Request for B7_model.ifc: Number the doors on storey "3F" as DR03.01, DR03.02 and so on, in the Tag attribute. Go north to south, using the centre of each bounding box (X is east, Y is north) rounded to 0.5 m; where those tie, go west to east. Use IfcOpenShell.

First a look at what the model holds.

```python
import ifcopenshell
import ifcopenshell.util.element
import ifcopenshell.util.placement

model = ifcopenshell.open("B7_model.ifc")
print(model.schema)
storey = next(s for s in model.by_type("IfcBuildingStorey") if s.Name == "3F")
doors = [e for e in ifcopenshell.util.element.get_decomposition(storey) if e.is_a("IfcDoor")]
for e in sorted(doors, key=lambda e: e.id()):
    origin = ifcopenshell.util.placement.get_local_placement(e.ObjectPlacement)[:3, 3]
    print(e.id(), e.Tag, e.Name, origin.round(2) + 0.0, sep=" | ")
```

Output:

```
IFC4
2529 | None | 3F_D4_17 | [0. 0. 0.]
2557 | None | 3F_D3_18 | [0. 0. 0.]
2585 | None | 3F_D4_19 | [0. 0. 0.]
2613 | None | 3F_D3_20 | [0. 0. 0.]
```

```python
import ifcopenshell
import ifcopenshell.geom
import ifcopenshell.util.element
import ifcopenshell.util.shape

model = ifcopenshell.open("B7_model.ifc")
settings = ifcopenshell.geom.settings()
settings.set("use-world-coords", True)


def centre(element):
    shape = ifcopenshell.geom.create_shape(settings, element)
    return ifcopenshell.util.shape.get_bbox_centroid(shape.geometry)


storey = next(s for s in model.by_type("IfcBuildingStorey") if s.Name == "3F")
doors = [e for e in ifcopenshell.util.element.get_decomposition(storey) if e.is_a("IfcDoor")]

# Insertion points can sit at a corner or the storey origin, so sort by the geometry (in metres).
centres = {e: centre(e) for e in doors}
doors.sort(key=lambda e: (-round(centres[e][1] / 0.5), centres[e][0]))

for i, e in enumerate(doors, start=1):
    number = f"DR03.{i:02d}"
    e.Tag = number
    print(e.id(), number)

model.write("B7_model_edited.ifc")
```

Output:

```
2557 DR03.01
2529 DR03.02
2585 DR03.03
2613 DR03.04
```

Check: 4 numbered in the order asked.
